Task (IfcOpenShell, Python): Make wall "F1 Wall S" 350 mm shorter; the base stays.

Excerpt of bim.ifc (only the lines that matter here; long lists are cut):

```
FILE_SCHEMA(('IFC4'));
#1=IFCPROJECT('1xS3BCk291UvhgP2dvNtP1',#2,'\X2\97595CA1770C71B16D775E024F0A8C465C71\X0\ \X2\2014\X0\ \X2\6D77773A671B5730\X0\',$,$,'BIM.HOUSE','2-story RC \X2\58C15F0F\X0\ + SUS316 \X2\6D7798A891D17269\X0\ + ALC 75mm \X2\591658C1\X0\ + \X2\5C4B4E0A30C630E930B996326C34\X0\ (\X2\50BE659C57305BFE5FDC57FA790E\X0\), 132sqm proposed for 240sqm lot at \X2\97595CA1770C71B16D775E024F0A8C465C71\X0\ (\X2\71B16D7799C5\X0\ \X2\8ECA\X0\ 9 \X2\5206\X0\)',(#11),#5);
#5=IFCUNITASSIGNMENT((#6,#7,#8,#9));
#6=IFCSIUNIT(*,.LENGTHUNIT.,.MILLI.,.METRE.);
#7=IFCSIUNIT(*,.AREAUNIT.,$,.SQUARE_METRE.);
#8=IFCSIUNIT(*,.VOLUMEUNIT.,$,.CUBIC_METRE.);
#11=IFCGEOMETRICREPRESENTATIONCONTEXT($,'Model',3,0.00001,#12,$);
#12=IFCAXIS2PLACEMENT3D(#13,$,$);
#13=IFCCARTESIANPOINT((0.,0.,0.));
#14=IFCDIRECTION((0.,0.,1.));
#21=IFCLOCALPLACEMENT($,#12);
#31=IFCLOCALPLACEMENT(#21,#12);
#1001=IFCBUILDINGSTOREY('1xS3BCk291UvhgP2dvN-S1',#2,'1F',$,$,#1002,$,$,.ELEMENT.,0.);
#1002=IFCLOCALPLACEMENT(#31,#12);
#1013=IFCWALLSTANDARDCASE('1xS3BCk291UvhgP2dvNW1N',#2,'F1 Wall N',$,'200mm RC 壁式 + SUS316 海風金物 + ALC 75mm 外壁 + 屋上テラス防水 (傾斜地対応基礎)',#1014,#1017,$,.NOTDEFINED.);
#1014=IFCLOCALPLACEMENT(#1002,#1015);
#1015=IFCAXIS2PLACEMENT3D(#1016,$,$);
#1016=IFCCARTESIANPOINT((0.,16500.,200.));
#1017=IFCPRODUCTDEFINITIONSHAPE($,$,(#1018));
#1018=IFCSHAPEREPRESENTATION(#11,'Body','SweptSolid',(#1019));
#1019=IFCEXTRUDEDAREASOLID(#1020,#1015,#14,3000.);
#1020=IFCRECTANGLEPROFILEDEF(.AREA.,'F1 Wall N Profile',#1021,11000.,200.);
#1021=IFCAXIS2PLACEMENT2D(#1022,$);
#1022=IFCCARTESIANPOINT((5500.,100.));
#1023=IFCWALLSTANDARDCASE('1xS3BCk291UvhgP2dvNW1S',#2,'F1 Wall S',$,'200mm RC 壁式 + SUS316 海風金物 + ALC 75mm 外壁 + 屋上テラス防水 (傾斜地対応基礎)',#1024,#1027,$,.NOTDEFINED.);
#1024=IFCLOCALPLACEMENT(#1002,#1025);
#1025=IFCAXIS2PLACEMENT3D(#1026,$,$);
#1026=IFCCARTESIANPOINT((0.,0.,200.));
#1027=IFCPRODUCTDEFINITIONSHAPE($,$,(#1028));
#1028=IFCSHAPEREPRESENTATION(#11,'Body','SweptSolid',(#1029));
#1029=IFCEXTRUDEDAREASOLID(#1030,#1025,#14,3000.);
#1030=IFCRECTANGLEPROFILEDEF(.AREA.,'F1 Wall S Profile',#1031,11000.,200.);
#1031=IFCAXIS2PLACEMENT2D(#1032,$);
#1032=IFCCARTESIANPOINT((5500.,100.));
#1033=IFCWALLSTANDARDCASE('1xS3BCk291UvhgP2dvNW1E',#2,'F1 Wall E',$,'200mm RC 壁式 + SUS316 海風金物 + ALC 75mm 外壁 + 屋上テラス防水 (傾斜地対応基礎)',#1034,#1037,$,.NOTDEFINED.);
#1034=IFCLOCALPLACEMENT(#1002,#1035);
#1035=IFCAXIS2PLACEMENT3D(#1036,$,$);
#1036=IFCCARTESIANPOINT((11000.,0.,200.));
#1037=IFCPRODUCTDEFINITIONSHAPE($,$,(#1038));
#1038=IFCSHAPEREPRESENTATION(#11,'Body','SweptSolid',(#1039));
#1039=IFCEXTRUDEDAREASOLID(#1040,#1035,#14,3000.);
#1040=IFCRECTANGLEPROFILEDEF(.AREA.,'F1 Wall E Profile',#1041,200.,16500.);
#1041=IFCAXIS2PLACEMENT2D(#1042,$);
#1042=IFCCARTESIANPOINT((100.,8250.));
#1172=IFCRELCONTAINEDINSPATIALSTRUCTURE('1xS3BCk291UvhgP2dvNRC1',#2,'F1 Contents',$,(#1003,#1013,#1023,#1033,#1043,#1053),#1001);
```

```python
import ifcopenshell
import ifcopenshell.geom
import ifcopenshell.util.shape

model = ifcopenshell.open("bim.ifc")
settings = ifcopenshell.geom.settings()


def volume(element):
    """Net volume in cubic metres, openings subtracted."""
    shape = ifcopenshell.geom.create_shape(settings, element)
    return ifcopenshell.util.shape.get_volume(shape.geometry)


wall = model.by_guid("1xS3BCk291UvhgP2dvNW1S")
before = volume(wall)

body = next(r for r in wall.Representation.Representations if r.RepresentationIdentifier == "Body")
solid = body.Items[0]
old_height = solid.Depth
solid.Depth -= 350.0
after = volume(wall)

print(f"height {old_height:g} -> {solid.Depth:g}, volume {before:.3f} -> {after:.3f} m3")

model.write("bim_v2.ifc")
```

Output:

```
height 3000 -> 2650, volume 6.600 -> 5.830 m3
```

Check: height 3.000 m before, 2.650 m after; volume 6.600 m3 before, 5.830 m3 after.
